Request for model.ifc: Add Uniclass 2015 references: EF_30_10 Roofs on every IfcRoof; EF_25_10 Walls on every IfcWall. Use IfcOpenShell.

First a look at what the model holds.

```python
import ifcopenshell

model = ifcopenshell.open("model.ifc")
print(model.schema)
print("classifications:", [c.Name for c in model.by_type("IfcClassification")])
for ifc_class in ("IfcDoor", "IfcRoof", "IfcStair", "IfcWall", "IfcWindow"):
    print(ifc_class, len(model.by_type(ifc_class)))
```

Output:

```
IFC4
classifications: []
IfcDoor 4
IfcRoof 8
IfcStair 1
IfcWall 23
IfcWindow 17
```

```python
import ifcopenshell
import ifcopenshell.api.classification

model = ifcopenshell.open("model.ifc")

system = ifcopenshell.api.classification.add_classification(model, classification="Uniclass 2015")

codes = {
    "IfcRoof": ("EF_30_10", "Roofs"),
    "IfcWall": ("EF_25_10", "Walls"),
}
for ifc_class, (code, name) in codes.items():
    products = model.by_type(ifc_class)
    ifcopenshell.api.classification.add_reference(
        model, products=products, classification=system, identification=code, name=name
    )
    print(code, len(products))

model.write("model-out.ifc")
```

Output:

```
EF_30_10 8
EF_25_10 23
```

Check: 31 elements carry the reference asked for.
